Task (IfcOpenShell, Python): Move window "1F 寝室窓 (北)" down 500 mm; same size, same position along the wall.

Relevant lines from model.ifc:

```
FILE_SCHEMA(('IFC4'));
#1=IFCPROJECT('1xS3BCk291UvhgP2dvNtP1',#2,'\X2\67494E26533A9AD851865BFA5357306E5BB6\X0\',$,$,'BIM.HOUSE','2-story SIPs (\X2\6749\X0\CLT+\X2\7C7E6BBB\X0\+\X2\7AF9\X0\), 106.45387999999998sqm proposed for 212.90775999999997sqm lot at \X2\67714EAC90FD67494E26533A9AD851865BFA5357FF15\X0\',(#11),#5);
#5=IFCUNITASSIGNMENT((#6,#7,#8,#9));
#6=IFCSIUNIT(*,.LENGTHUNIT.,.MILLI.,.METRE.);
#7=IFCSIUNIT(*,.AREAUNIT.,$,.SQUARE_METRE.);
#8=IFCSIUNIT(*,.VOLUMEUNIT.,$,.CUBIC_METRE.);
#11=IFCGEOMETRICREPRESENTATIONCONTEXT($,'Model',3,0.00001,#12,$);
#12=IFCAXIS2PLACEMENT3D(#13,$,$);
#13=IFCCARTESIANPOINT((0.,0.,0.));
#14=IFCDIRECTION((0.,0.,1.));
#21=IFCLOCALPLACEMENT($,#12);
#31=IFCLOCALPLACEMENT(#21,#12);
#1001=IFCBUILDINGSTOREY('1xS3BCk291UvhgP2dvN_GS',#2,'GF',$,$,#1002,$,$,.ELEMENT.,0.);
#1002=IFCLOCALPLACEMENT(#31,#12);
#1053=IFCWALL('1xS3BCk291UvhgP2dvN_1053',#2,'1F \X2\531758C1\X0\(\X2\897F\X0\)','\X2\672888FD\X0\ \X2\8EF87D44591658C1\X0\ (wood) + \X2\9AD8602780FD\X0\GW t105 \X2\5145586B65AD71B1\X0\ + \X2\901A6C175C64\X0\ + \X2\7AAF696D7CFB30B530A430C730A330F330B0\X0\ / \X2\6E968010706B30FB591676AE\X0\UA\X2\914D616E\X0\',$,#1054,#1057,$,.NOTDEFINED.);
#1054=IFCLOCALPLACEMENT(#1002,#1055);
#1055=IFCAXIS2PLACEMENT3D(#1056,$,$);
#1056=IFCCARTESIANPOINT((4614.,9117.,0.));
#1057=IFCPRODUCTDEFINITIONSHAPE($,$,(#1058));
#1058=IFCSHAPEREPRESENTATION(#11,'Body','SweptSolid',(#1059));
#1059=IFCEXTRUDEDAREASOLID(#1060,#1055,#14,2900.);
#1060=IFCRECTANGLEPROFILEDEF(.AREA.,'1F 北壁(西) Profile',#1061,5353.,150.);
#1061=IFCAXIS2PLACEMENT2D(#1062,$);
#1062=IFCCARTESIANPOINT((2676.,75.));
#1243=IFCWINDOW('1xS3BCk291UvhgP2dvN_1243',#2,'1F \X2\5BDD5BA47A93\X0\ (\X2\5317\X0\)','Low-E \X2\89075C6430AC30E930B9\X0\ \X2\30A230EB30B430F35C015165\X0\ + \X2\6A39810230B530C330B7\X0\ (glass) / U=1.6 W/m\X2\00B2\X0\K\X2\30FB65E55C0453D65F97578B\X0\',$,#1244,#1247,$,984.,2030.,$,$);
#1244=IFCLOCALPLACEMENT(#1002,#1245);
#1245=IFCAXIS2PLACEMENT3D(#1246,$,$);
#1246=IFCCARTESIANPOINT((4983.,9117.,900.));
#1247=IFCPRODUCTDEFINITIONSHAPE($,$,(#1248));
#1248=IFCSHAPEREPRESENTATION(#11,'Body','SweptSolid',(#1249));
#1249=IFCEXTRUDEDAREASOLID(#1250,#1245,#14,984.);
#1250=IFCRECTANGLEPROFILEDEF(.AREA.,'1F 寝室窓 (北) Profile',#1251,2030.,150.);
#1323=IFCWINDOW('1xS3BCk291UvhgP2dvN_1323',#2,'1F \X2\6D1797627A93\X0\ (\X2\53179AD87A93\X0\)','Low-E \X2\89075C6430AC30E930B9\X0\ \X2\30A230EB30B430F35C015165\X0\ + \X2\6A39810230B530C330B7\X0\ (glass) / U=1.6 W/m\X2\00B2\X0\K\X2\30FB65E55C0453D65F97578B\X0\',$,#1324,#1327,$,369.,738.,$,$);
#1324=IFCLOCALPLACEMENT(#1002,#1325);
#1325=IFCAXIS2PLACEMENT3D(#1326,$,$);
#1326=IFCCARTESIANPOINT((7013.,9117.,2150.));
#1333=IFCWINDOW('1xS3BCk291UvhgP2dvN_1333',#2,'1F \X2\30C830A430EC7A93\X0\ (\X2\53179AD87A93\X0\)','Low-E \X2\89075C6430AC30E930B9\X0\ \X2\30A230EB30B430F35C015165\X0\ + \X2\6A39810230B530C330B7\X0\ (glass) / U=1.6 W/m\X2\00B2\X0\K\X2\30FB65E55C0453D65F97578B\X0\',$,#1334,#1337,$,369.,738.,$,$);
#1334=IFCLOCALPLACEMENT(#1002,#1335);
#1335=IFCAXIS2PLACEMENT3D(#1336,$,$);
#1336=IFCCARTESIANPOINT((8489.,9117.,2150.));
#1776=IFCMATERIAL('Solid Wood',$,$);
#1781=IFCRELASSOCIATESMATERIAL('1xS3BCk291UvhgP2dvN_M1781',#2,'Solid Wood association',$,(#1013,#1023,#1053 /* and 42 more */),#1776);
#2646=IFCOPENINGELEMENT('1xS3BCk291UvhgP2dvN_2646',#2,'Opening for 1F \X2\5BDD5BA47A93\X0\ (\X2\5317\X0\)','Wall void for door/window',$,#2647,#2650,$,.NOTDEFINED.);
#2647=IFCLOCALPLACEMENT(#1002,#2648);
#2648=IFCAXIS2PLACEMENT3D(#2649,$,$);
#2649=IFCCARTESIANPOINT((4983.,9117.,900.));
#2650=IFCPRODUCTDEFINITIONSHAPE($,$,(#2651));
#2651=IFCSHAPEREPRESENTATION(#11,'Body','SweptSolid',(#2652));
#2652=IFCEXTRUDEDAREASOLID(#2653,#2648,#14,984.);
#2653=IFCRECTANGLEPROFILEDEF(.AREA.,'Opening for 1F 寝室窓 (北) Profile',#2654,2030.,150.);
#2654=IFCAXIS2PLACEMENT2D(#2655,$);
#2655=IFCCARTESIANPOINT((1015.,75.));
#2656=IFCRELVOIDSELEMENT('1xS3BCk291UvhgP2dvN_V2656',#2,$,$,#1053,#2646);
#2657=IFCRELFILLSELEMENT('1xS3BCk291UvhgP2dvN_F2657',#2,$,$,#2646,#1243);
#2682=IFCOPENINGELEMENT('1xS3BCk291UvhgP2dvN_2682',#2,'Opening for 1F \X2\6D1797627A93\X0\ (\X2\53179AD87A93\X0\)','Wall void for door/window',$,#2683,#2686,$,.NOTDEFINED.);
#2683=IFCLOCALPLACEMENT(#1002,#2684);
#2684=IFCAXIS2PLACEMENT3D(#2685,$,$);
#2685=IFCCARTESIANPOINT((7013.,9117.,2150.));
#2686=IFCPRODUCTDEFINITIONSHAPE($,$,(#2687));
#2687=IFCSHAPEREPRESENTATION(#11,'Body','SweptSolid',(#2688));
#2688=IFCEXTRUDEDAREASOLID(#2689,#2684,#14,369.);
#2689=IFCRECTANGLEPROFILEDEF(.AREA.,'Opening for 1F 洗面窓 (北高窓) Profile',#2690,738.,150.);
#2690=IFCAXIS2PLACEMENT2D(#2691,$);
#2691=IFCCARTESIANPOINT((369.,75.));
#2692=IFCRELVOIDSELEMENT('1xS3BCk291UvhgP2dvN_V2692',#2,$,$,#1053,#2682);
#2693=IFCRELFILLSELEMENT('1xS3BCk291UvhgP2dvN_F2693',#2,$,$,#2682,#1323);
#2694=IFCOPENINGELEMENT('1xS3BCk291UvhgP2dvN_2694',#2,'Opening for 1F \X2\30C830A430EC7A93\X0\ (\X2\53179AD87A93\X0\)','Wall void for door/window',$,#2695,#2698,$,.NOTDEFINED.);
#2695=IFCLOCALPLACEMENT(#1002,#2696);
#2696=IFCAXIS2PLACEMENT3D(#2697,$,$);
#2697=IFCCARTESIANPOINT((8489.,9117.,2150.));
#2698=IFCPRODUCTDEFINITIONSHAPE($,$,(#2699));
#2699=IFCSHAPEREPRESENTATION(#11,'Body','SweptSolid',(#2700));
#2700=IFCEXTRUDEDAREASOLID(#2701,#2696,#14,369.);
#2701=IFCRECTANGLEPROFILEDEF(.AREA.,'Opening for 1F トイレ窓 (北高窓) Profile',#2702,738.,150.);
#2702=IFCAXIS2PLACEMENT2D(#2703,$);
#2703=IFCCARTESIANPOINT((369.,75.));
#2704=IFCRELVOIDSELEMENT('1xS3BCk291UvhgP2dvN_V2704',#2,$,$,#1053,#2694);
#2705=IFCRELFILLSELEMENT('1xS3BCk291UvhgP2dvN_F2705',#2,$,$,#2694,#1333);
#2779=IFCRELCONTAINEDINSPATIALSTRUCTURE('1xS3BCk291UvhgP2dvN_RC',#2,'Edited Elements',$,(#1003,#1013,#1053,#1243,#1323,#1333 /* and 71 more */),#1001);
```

```python
import numpy as np
import ifcopenshell
import ifcopenshell.api.geometry
import ifcopenshell.util.placement
import ifcopenshell.util.unit

model = ifcopenshell.open("model.ifc")
unit_scale = ifcopenshell.util.unit.calculate_unit_scale(model)

window = model.by_guid("1xS3BCk291UvhgP2dvN_1243")
opening = window.FillsVoids[0].RelatingOpeningElement
dz = -0.5 / unit_scale

shift = np.array([0.0, 0.0, dz])
# The window is not placed relative to its opening, so move both.
for product in (opening, window):
    matrix = ifcopenshell.util.placement.get_local_placement(product.ObjectPlacement)
    matrix[:3, 3] += shift
    ifcopenshell.api.geometry.edit_object_placement(model, product=product, matrix=matrix, is_si=False)

print(f"moved by {dz * unit_scale:+.3f} m")

model.write("model-out.ifc")
```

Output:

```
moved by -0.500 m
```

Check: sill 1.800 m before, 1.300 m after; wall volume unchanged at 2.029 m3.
